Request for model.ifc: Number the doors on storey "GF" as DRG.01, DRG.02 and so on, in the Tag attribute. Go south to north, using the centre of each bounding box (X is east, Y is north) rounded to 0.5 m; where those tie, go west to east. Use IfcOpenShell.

First a look at what the model holds.

```python
import ifcopenshell
import ifcopenshell.util.element
import ifcopenshell.util.placement

model = ifcopenshell.open("model.ifc")
print(model.schema)
storey = next(s for s in model.by_type("IfcBuildingStorey") if s.Name == "GF")
doors = [e for e in ifcopenshell.util.element.get_decomposition(storey) if e.is_a("IfcDoor")]
for e in sorted(doors, key=lambda e: e.id()):
    origin = ifcopenshell.util.placement.get_local_placement(e.ObjectPlacement)[:3, 3]
    print(e.id(), e.Tag, e.Name, origin.round(2) + 0.0, sep=" | ")
```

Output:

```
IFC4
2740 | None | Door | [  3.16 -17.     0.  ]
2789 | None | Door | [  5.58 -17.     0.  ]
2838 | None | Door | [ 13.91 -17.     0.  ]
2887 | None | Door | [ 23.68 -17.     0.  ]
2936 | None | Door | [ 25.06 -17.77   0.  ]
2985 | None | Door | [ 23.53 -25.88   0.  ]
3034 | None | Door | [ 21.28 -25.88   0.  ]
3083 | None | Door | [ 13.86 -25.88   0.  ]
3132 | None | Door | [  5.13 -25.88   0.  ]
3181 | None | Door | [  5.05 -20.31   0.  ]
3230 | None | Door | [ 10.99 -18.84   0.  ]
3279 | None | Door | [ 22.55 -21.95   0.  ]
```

```python
import ifcopenshell
import ifcopenshell.geom
import ifcopenshell.util.element
import ifcopenshell.util.shape

model = ifcopenshell.open("model.ifc")
settings = ifcopenshell.geom.settings()
settings.set("use-world-coords", True)


def centre(element):
    shape = ifcopenshell.geom.create_shape(settings, element)
    return ifcopenshell.util.shape.get_bbox_centroid(shape.geometry)


storey = next(s for s in model.by_type("IfcBuildingStorey") if s.Name == "GF")
doors = [e for e in ifcopenshell.util.element.get_decomposition(storey) if e.is_a("IfcDoor")]

# Insertion points can sit at a corner or the storey origin, so sort by the geometry (in metres).
centres = {e: centre(e) for e in doors}
doors.sort(key=lambda e: (round(centres[e][1] / 0.5), centres[e][0]))

for i, e in enumerate(doors, start=1):
    number = f"DRG.{i:02d}"
    e.Tag = number
    print(e.id(), number)

model.write("model_edited.ifc")
```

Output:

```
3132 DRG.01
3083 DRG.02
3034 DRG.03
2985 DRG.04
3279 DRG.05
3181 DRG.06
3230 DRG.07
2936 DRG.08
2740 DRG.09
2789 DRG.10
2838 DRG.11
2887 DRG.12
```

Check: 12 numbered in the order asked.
